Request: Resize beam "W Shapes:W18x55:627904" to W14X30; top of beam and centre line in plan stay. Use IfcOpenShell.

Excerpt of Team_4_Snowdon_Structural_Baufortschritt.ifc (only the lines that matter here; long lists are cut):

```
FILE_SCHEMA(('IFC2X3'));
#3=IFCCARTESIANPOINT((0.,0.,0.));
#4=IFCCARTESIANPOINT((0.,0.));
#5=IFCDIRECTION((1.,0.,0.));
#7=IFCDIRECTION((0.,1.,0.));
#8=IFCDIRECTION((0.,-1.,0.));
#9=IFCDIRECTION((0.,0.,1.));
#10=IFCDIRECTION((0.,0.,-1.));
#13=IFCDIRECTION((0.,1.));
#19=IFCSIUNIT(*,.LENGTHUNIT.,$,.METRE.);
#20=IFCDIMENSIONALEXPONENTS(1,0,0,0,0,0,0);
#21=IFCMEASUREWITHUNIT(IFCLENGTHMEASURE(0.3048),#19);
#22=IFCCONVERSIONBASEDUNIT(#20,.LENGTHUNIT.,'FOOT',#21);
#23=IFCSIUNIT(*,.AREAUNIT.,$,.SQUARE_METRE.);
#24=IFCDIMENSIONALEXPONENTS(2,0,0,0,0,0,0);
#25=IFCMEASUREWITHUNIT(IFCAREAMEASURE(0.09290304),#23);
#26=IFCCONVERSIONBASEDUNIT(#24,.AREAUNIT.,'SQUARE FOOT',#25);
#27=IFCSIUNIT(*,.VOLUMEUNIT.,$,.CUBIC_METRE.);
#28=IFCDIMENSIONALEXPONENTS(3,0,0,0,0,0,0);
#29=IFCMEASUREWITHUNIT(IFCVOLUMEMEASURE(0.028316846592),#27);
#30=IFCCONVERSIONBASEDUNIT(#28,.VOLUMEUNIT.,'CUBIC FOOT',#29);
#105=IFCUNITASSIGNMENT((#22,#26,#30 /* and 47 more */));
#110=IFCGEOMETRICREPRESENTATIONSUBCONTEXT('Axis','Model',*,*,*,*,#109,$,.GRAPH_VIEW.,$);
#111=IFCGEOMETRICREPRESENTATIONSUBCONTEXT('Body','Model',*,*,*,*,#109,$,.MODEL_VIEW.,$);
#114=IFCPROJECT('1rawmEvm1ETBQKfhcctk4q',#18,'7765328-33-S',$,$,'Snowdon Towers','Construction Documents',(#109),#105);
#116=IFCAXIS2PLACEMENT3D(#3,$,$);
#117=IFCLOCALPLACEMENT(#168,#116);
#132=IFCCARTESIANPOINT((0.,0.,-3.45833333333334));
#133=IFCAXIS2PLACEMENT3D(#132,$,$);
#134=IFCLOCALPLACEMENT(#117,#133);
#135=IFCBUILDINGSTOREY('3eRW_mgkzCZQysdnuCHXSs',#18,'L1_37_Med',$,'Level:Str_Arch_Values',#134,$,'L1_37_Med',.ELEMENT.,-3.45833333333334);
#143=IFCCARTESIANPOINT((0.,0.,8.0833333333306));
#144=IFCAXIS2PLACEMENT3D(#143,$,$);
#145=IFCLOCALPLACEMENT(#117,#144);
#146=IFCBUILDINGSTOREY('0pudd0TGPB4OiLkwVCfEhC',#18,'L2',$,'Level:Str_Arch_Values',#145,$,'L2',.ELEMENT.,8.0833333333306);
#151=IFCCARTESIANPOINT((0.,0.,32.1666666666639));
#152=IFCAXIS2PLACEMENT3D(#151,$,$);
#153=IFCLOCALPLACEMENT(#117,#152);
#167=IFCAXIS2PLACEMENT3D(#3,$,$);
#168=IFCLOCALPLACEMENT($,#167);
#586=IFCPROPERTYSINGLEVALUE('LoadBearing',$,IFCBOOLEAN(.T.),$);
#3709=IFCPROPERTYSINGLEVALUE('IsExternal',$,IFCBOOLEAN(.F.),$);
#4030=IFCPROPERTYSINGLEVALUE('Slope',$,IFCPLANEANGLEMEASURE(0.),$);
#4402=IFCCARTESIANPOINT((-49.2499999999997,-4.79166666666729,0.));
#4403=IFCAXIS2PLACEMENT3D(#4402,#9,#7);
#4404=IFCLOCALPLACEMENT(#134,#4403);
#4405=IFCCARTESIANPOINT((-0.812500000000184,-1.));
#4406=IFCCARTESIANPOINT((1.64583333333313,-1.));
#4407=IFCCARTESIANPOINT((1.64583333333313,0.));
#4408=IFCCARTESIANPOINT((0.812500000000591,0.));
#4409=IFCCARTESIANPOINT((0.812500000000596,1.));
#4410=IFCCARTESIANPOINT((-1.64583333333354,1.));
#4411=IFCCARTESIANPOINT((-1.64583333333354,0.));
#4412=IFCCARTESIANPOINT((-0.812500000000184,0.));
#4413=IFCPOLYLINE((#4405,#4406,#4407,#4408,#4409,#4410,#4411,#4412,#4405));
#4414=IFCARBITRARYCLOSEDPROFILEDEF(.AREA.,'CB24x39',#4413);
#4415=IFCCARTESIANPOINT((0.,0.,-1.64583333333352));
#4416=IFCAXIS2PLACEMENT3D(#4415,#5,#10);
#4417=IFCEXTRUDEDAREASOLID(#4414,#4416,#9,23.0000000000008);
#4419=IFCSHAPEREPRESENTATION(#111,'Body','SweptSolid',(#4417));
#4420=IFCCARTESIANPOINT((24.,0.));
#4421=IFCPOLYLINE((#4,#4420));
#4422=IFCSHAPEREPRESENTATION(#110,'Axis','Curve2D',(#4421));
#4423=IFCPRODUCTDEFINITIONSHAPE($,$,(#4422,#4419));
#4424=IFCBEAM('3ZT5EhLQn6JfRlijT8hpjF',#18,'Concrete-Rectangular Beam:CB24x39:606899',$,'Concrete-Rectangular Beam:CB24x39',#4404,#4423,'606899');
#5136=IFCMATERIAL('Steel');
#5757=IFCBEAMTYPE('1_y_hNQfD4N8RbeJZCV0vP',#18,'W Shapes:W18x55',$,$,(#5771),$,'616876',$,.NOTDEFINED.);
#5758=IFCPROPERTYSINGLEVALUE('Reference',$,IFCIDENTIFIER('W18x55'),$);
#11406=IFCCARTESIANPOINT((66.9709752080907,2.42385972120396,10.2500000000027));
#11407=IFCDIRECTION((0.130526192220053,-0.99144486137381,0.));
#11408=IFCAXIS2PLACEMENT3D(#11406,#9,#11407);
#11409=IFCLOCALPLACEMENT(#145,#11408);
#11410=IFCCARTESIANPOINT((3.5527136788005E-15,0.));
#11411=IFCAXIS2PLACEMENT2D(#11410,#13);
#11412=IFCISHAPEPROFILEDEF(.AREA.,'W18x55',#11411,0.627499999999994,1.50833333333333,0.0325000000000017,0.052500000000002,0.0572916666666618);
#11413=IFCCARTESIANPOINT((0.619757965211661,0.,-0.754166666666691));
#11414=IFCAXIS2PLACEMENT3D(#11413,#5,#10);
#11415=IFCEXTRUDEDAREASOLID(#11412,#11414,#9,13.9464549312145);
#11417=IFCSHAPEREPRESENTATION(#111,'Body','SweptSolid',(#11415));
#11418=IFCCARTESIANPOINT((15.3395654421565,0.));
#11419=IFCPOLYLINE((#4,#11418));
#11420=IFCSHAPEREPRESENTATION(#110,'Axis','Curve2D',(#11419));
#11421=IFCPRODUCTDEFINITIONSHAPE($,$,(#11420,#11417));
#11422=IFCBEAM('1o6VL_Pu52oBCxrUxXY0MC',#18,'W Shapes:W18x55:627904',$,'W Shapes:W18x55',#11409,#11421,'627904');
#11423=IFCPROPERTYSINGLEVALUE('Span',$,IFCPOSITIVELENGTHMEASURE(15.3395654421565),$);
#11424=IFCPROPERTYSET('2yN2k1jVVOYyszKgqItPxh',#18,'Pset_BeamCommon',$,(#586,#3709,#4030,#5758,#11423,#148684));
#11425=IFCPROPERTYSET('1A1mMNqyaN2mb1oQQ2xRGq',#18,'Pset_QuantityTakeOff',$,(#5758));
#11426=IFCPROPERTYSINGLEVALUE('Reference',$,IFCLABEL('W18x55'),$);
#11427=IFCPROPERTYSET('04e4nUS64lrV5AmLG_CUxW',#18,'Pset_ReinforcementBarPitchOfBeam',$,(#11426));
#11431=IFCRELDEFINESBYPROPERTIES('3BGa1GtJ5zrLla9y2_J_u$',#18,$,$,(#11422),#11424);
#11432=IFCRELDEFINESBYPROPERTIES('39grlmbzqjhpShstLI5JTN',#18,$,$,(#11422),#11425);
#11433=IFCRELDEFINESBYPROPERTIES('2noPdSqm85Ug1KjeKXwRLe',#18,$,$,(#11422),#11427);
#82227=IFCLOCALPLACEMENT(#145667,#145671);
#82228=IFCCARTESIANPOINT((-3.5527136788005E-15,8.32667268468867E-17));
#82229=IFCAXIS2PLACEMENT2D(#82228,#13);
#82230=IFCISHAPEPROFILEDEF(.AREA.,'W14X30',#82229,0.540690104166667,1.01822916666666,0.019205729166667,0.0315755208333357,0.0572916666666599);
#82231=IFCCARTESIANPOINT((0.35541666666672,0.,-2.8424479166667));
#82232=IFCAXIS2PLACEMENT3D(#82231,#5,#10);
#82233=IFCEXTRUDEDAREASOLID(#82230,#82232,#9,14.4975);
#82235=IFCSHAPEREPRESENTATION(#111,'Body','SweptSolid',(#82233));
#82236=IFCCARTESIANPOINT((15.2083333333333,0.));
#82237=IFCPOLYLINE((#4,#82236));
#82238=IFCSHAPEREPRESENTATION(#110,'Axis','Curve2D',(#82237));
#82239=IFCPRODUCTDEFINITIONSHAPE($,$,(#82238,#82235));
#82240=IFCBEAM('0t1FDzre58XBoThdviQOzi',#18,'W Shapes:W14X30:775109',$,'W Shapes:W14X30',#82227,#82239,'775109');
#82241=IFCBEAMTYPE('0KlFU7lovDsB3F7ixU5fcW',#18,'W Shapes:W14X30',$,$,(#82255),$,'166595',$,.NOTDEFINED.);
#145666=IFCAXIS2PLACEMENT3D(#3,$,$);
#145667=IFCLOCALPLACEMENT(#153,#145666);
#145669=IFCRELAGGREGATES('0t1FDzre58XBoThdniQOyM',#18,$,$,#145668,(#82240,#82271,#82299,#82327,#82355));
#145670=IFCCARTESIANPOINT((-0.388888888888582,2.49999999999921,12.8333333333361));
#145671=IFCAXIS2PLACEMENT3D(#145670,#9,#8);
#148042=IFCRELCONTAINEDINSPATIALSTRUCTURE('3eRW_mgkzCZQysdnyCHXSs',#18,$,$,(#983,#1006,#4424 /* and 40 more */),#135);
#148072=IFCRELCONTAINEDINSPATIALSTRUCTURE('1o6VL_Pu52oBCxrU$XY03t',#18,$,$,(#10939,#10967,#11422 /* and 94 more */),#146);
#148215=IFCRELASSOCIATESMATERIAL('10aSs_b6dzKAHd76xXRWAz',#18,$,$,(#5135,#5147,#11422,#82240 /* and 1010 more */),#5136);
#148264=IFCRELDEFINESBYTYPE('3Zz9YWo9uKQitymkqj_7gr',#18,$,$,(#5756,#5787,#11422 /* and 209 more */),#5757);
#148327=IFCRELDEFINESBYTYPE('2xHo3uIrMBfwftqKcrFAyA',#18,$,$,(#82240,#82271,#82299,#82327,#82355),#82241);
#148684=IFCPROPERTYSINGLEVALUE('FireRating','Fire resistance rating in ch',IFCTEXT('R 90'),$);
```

```python
import ifcopenshell
import ifcopenshell.api.pset
import ifcopenshell.api.type
import ifcopenshell.util.element
import ifcopenshell.util.representation

model = ifcopenshell.open("Team_4_Snowdon_Structural_Baufortschritt.ifc")

member = model.by_id(11422)
source = next(p for p in model.by_type("IfcIShapeProfileDef") if p.ProfileName == "W14X30")

body = ifcopenshell.util.representation.get_representation(member, "Model", "Body")
solid = body.Items[0]
old_profile = solid.SweptArea

# Copy the section's sizes but keep this member's own profile position.
profile = ifcopenshell.util.element.copy(model, source)
# Profiles are centred, so shift by half the change in depth to hold the top.
shift = (old_profile.OverallDepth - profile.OverallDepth) / 2
x, y = old_profile.Position.Location.Coordinates
up = (-1.0, 0.0)  # upwards, in the solid's own plane
location = model.createIfcCartesianPoint((x + up[0] * shift, y + up[1] * shift))
profile.Position = model.createIfcAxis2Placement2D(location, old_profile.Position.RefDirection)
solid.SweptArea = profile
if not model.get_total_inverses(old_profile):
    ifcopenshell.util.element.remove_deep2(model, old_profile)

new_type = model.by_guid("0KlFU7lovDsB3F7ixU5fcW")
ifcopenshell.api.type.assign_type(
    model, related_objects=[member], relating_type=new_type, should_map_representations=False
)
member.Name = member.Name.replace("W18x55", "W14X30")
member.ObjectType = "W Shapes:W14X30"
pset = model.by_id(ifcopenshell.util.element.get_pset(member, "Pset_BeamCommon", should_inherit=False)["id"])
ifcopenshell.api.pset.edit_pset(model, pset=pset, properties={"Reference": "W14X30"})
pset = model.by_id(ifcopenshell.util.element.get_pset(member, "Pset_QuantityTakeOff", should_inherit=False)["id"])
ifcopenshell.api.pset.edit_pset(model, pset=pset, properties={"Reference": "W14X30"})
pset = model.by_id(ifcopenshell.util.element.get_pset(member, "Pset_ReinforcementBarPitchOfBeam", should_inherit=False)["id"])
ifcopenshell.api.pset.edit_pset(model, pset=pset, properties={"Reference": "W14X30"})

print(solid.SweptArea)

model.write("Team_4_Snowdon_Structural_Baufortschritt_updated.ifc")
```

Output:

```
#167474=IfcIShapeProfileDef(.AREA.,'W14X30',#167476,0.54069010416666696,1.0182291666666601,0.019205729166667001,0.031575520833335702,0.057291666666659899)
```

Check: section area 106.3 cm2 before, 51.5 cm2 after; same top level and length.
